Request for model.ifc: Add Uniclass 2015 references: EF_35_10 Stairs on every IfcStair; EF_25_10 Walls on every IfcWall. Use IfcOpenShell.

First a look at what the model holds.

```python
import ifcopenshell

model = ifcopenshell.open("model.ifc")
print(model.schema)
print("classifications:", [c.Name for c in model.by_type("IfcClassification")])
for ifc_class in ("IfcDoor", "IfcRoof", "IfcStair", "IfcWall", "IfcWindow"):
    print(ifc_class, len(model.by_type(ifc_class)))
```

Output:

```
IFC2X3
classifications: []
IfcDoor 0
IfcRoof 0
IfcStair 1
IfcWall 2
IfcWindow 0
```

```python
import ifcopenshell
import ifcopenshell.api.classification

model = ifcopenshell.open("model.ifc")

# IFC2X3 requires Source and Edition and has no link from the project to the system.
system = model.create_entity("IfcClassification", Source="NBS", Edition="2015", Name="Uniclass 2015")

codes = {
    "IfcStair": ("EF_35_10", "Stairs"),
    "IfcWall": ("EF_25_10", "Walls"),
}
for ifc_class, (code, name) in codes.items():
    products = model.by_type(ifc_class)
    ifcopenshell.api.classification.add_reference(
        model, products=products, classification=system, identification=code, name=name
    )
    print(code, len(products))

model.write("model-out.ifc")
```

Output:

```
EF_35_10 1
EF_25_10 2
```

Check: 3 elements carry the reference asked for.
